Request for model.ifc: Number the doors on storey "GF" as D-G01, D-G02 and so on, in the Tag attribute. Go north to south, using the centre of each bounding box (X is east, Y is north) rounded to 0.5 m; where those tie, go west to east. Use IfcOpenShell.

First a look at what the model holds.

```python
import ifcopenshell
import ifcopenshell.util.element
import ifcopenshell.util.placement

model = ifcopenshell.open("model.ifc")
print(model.schema)
storey = next(s for s in model.by_type("IfcBuildingStorey") if s.Name == "GF")
doors = [e for e in ifcopenshell.util.element.get_decomposition(storey) if e.is_a("IfcDoor")]
for e in sorted(doors, key=lambda e: e.id()):
    origin = ifcopenshell.util.placement.get_local_placement(e.ObjectPlacement)[:3, 3]
    print(e.id(), e.Tag, e.Name, origin.round(2) + 0.0, sep=" | ")
```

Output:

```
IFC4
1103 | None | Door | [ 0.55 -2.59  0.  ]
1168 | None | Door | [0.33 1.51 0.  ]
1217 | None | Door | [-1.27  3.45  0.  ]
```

```python
import ifcopenshell
import ifcopenshell.geom
import ifcopenshell.util.element
import ifcopenshell.util.shape

model = ifcopenshell.open("model.ifc")
settings = ifcopenshell.geom.settings()
settings.set("use-world-coords", True)


def centre(element):
    shape = ifcopenshell.geom.create_shape(settings, element)
    return ifcopenshell.util.shape.get_bbox_centroid(shape.geometry)


storey = next(s for s in model.by_type("IfcBuildingStorey") if s.Name == "GF")
doors = [e for e in ifcopenshell.util.element.get_decomposition(storey) if e.is_a("IfcDoor")]

# Insertion points can sit at a corner or the storey origin, so sort by the geometry (in metres).
centres = {e: centre(e) for e in doors}
doors.sort(key=lambda e: (-round(centres[e][1] / 0.5), centres[e][0]))

for i, e in enumerate(doors, start=1):
    number = f"D-G{i:02d}"
    e.Tag = number
    print(e.id(), number)

model.write("model_updated.ifc")
```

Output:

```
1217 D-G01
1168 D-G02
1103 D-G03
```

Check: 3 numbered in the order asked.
